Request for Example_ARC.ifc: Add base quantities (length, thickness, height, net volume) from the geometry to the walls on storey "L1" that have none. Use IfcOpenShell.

First a look at what the model holds.

```python
import ifcopenshell
import ifcopenshell.util.element
import ifcopenshell.util.unit

model = ifcopenshell.open("Example_ARC.ifc")
print(model.schema)
for unit_type in ("LENGTHUNIT", "AREAUNIT", "VOLUMEUNIT"):
    print(unit_type, ifcopenshell.util.unit.calculate_unit_scale(model, unit_type))
storey = next(s for s in model.by_type("IfcBuildingStorey") if s.Name == "L1")
walls = [e for e in ifcopenshell.util.element.get_decomposition(storey) if e.is_a("IfcWall")]
for e in sorted(walls, key=lambda e: e.id()):
    print(e.id(), e.is_a(), e.Name, list(ifcopenshell.util.element.get_psets(e, qtos_only=True)), sep=" | ")
```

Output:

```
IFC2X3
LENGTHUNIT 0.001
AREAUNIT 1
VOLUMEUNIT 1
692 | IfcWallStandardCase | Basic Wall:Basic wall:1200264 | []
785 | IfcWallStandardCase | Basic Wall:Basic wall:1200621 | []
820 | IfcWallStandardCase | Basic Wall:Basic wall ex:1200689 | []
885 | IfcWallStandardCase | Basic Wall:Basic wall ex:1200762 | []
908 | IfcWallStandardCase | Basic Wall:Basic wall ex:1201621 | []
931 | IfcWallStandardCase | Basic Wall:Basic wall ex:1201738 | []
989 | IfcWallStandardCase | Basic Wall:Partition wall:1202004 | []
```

```python
import ifcopenshell
import ifcopenshell.api.pset
import ifcopenshell.geom
import ifcopenshell.util.element
import ifcopenshell.util.shape
import ifcopenshell.util.unit

model = ifcopenshell.open("Example_ARC.ifc")
unit_scale = ifcopenshell.util.unit.calculate_unit_scale(model)
volume_scale = ifcopenshell.util.unit.calculate_unit_scale(model, "VOLUMEUNIT")
settings = ifcopenshell.geom.settings()

storey = next(s for s in model.by_type("IfcBuildingStorey") if s.Name == "L1")
walls = [e for e in ifcopenshell.util.element.get_decomposition(storey) if e.is_a("IfcWall")]

for e in sorted(walls, key=lambda e: e.id()):
    if ifcopenshell.util.element.get_psets(e, qtos_only=True, should_inherit=False):
        continue
    # Geometry comes back in metres, in the element's own axes.
    shape = ifcopenshell.geom.create_shape(settings, e)
    values = {
        "Length": ifcopenshell.util.shape.get_x(shape.geometry) / unit_scale,
        "Width": ifcopenshell.util.shape.get_y(shape.geometry) / unit_scale,
        "Height": ifcopenshell.util.shape.get_z(shape.geometry) / unit_scale,
        "NetVolume": ifcopenshell.util.shape.get_volume(shape.geometry) / volume_scale,
    }
    qto = ifcopenshell.api.pset.add_qto(model, product=e, name="BaseQuantities")
    ifcopenshell.api.pset.edit_qto(model, qto=qto, properties=values)
    print(e.id(), {k: round(v, 3) for k, v in values.items()})

model.write("Example_ARC_v2.ifc")
```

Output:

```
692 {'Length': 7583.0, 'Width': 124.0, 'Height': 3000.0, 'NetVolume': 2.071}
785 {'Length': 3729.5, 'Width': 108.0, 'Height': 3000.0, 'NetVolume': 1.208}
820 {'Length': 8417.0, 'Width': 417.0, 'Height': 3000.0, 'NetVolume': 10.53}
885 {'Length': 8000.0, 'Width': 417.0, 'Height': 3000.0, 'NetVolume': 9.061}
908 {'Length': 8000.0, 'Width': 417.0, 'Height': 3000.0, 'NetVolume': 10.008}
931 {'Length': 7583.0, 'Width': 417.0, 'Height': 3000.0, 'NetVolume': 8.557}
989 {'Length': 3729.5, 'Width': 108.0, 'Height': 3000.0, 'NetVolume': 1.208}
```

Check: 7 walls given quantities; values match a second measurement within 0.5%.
